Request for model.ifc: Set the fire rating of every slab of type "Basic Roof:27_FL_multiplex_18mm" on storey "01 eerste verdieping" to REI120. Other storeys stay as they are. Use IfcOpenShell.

First a look at what the model holds.

```python
import ifcopenshell
import ifcopenshell.util.element

model = ifcopenshell.open("model.ifc")
print(model.schema)
storey = next(s for s in model.by_type("IfcBuildingStorey") if s.Name == "01 eerste verdieping")
slabs = [e for e in ifcopenshell.util.element.get_decomposition(storey) if e.is_a("IfcSlab")]
seen = {}
for e in slabs:
    element_type = ifcopenshell.util.element.get_type(e)
    key = (element_type.Name if element_type != e and element_type else None, ifcopenshell.util.element.get_pset(e, "Pset_SlabCommon", "FireRating"))
    seen[key] = seen.get(key, 0) + 1
for (name, value), count in sorted(seen.items(), key=str):
    print(count, "x", name, "|", value)
```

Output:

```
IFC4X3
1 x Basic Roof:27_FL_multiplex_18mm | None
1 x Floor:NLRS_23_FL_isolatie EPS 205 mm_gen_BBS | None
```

```python
import ifcopenshell
import ifcopenshell.api.pset
import ifcopenshell.util.element

model = ifcopenshell.open("model.ifc")

storey = next(s for s in model.by_type("IfcBuildingStorey") if s.Name == "01 eerste verdieping")
slabs = [e for e in ifcopenshell.util.element.get_decomposition(storey) if e.is_a("IfcSlab")]

count = 0
for e in slabs:
    element_type = ifcopenshell.util.element.get_type(e)
    if element_type in (None, e) or element_type.Name != "Basic Roof:27_FL_multiplex_18mm":
        continue
    # add_pset returns the element's existing set when there is one.
    pset = ifcopenshell.api.pset.add_pset(model, product=e, name="Pset_SlabCommon")
    ifcopenshell.api.pset.edit_pset(model, pset=pset, properties={"FireRating": "REI120"})
    count += 1

print(count, "slabs updated")

model.write("model-out.ifc")
```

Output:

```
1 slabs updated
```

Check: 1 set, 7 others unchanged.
